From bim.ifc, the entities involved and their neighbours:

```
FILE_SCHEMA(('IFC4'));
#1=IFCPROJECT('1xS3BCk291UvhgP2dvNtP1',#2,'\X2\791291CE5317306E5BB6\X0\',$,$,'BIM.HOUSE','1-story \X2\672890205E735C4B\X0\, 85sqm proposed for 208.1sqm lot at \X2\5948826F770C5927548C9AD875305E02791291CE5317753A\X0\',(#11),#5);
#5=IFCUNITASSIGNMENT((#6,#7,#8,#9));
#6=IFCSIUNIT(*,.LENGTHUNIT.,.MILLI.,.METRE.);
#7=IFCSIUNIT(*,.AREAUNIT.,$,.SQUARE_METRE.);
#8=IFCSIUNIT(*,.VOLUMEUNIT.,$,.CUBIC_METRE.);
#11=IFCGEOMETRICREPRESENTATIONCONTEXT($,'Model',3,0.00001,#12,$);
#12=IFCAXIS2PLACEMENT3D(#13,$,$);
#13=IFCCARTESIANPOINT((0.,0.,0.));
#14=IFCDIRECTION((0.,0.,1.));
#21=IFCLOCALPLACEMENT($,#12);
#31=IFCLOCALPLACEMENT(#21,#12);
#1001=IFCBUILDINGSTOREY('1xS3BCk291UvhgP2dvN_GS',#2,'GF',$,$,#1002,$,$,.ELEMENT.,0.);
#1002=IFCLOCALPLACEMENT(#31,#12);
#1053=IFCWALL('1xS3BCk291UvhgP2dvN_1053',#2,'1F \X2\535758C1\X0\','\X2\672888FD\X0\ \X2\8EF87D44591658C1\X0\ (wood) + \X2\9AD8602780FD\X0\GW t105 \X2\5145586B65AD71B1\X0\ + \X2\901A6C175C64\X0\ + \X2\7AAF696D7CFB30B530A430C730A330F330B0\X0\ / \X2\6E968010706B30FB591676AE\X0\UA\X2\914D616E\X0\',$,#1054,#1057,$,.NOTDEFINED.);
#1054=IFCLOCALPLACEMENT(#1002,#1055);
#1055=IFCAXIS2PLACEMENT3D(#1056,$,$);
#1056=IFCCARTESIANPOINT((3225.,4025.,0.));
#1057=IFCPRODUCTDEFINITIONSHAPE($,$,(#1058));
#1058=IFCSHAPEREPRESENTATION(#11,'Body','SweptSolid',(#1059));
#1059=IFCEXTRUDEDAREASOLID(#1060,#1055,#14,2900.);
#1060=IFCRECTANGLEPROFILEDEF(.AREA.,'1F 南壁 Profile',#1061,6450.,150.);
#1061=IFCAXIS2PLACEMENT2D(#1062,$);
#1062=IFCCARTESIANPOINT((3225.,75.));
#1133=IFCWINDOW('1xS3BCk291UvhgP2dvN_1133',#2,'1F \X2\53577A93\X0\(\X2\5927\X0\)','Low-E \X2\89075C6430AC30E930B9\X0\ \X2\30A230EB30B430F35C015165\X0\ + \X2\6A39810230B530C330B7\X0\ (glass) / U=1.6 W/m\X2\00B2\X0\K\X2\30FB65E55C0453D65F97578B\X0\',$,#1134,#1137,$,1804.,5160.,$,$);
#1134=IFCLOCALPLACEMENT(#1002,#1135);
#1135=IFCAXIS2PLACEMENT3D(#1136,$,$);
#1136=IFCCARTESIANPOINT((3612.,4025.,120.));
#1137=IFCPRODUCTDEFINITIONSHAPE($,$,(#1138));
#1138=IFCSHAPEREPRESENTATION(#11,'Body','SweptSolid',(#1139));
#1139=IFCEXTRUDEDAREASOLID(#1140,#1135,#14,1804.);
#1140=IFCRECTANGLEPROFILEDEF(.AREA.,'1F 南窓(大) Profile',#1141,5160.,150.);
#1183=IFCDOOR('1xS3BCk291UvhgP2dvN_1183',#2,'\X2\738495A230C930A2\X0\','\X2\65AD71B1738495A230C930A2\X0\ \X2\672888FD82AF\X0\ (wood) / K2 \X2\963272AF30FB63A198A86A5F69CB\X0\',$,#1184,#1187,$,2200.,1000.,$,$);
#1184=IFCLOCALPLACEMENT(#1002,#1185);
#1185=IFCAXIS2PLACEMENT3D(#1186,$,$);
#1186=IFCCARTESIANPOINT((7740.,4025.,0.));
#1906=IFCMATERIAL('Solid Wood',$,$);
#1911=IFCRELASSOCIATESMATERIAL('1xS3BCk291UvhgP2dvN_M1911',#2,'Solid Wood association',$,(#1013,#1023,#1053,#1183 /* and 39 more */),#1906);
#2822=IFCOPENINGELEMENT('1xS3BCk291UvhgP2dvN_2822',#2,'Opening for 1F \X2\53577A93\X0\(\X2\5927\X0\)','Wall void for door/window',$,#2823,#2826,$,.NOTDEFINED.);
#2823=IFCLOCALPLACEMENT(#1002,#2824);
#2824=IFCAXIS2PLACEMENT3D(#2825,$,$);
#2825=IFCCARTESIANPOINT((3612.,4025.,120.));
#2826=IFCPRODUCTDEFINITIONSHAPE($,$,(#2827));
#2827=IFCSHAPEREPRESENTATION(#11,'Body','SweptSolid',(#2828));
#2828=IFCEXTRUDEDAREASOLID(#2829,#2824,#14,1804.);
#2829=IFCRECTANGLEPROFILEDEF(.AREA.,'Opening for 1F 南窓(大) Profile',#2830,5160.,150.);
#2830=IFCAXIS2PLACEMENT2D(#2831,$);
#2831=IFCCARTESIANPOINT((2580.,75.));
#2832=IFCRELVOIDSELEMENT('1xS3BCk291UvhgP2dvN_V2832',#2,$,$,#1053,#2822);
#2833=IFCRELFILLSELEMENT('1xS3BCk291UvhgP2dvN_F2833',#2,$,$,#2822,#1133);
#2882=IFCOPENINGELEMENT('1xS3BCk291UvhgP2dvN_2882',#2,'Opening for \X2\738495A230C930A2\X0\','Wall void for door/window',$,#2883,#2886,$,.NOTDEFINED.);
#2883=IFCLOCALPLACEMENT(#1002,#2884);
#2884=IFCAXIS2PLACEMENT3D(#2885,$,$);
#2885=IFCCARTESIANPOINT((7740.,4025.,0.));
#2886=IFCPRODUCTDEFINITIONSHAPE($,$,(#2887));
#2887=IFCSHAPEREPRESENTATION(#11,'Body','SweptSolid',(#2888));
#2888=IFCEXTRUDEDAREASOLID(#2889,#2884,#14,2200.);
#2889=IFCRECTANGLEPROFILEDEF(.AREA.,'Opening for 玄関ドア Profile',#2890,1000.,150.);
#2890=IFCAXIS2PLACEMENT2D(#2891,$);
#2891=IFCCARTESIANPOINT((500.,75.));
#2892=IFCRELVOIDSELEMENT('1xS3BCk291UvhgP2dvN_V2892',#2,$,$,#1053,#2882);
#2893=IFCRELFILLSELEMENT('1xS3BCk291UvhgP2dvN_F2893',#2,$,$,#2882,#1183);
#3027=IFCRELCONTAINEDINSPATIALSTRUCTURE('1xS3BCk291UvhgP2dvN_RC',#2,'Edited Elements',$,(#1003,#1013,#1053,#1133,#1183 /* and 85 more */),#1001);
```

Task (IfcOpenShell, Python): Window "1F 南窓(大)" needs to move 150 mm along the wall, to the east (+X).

```python
import ifcopenshell
import ifcopenshell.api.geometry
import ifcopenshell.util.placement

model = ifcopenshell.open("bim.ifc")

window = model.by_guid("1xS3BCk291UvhgP2dvN_1133")
opening = window.FillsVoids[0].RelatingOpeningElement
wall = opening.VoidsElements[0].RelatingBuildingElement

wall_matrix = ifcopenshell.util.placement.get_local_placement(wall.ObjectPlacement)
shift = wall_matrix[:3, 0] * 150.0
before = ifcopenshell.util.placement.get_local_placement(window.ObjectPlacement)[:3, 3].copy()

# The window is not placed relative to its opening, so move both.
for product in (opening, window):
    matrix = ifcopenshell.util.placement.get_local_placement(product.ObjectPlacement)
    matrix[:3, 3] += shift
    ifcopenshell.api.geometry.edit_object_placement(model, product=product, matrix=matrix, is_si=False)

after = ifcopenshell.util.placement.get_local_placement(window.ObjectPlacement)[:3, 3]
print("window moved by", (after - before).round(3) + 0.0)

model.write("bim_edited.ifc")
```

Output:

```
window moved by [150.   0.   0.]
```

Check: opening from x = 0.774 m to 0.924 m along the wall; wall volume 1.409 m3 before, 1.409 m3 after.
